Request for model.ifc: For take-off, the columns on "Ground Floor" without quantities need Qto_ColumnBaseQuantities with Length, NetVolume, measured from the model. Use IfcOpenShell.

First a look at what the model holds.

```python
import ifcopenshell
import ifcopenshell.util.element
import ifcopenshell.util.unit

model = ifcopenshell.open("model.ifc")
print(model.schema)
for unit_type in ("LENGTHUNIT", "AREAUNIT", "VOLUMEUNIT"):
    print(unit_type, ifcopenshell.util.unit.calculate_unit_scale(model, unit_type))
storey = next(s for s in model.by_type("IfcBuildingStorey") if s.Name == "Ground Floor")
columns = [e for e in ifcopenshell.util.element.get_decomposition(storey) if e.is_a("IfcColumn")]
for e in sorted(columns, key=lambda e: e.id()):
    print(e.id(), e.is_a(), e.Name, list(ifcopenshell.util.element.get_psets(e, qtos_only=True)), sep=" | ")
```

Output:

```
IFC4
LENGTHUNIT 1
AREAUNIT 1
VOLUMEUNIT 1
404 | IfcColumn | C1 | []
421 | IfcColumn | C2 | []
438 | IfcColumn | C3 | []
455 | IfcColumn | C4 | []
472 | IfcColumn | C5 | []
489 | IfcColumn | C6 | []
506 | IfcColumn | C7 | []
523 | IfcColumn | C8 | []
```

```python
import ifcopenshell
import ifcopenshell.api.pset
import ifcopenshell.geom
import ifcopenshell.util.element
import ifcopenshell.util.shape
import ifcopenshell.util.unit

model = ifcopenshell.open("model.ifc")
unit_scale = ifcopenshell.util.unit.calculate_unit_scale(model)
volume_scale = ifcopenshell.util.unit.calculate_unit_scale(model, "VOLUMEUNIT")
settings = ifcopenshell.geom.settings()

storey = next(s for s in model.by_type("IfcBuildingStorey") if s.Name == "Ground Floor")
columns = [e for e in ifcopenshell.util.element.get_decomposition(storey) if e.is_a("IfcColumn")]

for e in sorted(columns, key=lambda e: e.id()):
    if ifcopenshell.util.element.get_psets(e, qtos_only=True, should_inherit=False):
        continue
    # Geometry comes back in metres, in the element's own axes.
    shape = ifcopenshell.geom.create_shape(settings, e)
    values = {
        "Length": ifcopenshell.util.shape.get_z(shape.geometry) / unit_scale,
        "NetVolume": ifcopenshell.util.shape.get_volume(shape.geometry) / volume_scale,
    }
    qto = ifcopenshell.api.pset.add_qto(model, product=e, name="Qto_ColumnBaseQuantities")
    ifcopenshell.api.pset.edit_qto(model, qto=qto, properties=values)
    print(e.id(), {k: round(v, 3) for k, v in values.items()})

model.write("model_edited.ifc")
```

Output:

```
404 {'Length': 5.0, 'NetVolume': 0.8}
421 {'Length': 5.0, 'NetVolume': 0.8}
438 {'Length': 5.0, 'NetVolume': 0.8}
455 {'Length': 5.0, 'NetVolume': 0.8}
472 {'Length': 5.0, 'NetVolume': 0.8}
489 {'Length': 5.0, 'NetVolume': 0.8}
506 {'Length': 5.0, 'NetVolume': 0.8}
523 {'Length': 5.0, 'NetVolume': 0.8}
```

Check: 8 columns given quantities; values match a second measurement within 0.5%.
